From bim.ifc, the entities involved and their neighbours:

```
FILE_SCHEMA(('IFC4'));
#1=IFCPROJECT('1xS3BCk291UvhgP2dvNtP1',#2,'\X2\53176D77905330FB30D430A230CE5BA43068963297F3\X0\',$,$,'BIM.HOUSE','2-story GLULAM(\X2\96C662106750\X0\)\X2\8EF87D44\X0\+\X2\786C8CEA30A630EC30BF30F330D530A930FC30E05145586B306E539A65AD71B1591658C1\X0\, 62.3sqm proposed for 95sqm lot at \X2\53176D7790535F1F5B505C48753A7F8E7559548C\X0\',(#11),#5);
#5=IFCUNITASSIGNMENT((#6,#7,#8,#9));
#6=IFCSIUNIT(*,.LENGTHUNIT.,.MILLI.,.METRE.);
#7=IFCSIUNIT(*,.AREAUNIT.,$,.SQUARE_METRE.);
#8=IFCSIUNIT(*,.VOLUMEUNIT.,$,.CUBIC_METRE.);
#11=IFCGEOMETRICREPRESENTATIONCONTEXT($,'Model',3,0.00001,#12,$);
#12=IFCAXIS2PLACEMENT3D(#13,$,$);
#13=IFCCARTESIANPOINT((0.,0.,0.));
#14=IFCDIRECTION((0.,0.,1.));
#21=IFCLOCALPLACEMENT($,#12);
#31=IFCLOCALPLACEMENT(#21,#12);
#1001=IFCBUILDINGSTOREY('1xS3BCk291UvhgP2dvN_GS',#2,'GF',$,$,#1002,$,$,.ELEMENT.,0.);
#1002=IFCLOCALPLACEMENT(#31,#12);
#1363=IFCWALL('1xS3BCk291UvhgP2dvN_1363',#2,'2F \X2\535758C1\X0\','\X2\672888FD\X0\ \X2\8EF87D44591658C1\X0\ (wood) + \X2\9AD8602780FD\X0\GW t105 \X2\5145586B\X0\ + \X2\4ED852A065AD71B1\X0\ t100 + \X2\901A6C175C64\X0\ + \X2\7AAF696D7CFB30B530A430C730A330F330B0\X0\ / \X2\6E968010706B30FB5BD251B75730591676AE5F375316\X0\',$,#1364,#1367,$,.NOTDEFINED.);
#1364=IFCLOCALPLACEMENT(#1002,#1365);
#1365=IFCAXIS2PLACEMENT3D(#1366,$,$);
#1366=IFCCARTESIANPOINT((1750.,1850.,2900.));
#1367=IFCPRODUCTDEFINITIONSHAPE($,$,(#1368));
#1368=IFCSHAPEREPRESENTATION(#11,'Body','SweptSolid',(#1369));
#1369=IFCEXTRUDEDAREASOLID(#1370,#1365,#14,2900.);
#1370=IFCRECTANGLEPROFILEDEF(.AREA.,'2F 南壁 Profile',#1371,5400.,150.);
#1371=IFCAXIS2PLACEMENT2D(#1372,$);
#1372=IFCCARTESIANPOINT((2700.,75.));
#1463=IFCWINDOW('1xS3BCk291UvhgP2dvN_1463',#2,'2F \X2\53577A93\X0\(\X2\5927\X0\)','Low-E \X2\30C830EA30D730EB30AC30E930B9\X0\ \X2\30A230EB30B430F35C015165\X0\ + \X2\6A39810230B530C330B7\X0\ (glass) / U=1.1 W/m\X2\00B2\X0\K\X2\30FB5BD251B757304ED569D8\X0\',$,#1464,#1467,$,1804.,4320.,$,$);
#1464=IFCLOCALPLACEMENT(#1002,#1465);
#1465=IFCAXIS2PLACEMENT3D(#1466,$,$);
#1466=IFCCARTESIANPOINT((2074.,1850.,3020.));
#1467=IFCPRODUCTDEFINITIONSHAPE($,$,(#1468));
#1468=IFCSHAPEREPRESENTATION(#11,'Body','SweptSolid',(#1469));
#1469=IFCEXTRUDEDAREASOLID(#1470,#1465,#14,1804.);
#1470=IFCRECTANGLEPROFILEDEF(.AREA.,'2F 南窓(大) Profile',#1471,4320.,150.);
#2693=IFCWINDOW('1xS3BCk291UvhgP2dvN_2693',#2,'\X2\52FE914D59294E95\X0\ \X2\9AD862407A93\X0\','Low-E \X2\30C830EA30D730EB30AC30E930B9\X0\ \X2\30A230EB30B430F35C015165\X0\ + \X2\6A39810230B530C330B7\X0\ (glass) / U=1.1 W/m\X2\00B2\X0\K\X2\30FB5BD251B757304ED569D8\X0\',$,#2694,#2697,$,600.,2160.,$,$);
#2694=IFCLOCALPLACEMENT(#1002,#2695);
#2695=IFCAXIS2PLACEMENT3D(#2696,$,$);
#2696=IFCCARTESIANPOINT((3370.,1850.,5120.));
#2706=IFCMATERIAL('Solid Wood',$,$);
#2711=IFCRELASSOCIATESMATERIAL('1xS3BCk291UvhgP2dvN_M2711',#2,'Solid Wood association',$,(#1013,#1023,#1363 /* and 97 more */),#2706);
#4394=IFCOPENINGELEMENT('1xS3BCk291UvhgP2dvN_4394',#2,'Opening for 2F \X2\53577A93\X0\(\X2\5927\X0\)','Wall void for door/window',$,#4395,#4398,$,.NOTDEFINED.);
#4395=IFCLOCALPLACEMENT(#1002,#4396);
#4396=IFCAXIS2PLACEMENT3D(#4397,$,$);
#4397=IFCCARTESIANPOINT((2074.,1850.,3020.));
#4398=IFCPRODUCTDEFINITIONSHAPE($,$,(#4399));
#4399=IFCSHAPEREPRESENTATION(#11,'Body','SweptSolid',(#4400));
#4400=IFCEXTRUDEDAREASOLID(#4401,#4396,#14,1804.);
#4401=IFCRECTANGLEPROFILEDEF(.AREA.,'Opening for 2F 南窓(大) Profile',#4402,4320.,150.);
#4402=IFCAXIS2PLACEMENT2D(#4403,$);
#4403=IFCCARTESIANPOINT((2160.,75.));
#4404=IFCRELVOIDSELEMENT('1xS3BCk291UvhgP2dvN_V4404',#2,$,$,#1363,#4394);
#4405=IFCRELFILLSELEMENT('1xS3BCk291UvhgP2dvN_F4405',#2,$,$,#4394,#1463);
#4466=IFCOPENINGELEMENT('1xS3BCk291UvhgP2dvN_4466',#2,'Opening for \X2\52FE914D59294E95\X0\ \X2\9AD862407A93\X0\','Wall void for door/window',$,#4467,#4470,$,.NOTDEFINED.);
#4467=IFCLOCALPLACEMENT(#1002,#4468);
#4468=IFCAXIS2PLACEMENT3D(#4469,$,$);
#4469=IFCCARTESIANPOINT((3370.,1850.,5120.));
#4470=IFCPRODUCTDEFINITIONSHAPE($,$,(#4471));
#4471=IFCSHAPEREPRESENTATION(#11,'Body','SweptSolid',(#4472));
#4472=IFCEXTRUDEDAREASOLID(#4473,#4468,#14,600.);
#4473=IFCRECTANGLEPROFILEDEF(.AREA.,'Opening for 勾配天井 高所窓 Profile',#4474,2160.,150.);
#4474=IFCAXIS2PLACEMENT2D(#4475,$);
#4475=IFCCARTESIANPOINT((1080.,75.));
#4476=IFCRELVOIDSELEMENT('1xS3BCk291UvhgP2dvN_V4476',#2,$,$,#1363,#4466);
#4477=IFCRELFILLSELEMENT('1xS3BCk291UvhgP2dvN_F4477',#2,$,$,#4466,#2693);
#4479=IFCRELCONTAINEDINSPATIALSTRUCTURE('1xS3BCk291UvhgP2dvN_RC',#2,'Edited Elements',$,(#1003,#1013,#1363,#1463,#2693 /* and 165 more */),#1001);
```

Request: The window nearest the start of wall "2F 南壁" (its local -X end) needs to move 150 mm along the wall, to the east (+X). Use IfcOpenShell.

```python
import ifcopenshell
import ifcopenshell.api.geometry
import ifcopenshell.util.placement
import ifcopenshell.util.unit

model = ifcopenshell.open("bim.ifc")
unit_scale = ifcopenshell.util.unit.calculate_unit_scale(model)

window = model.by_guid("1xS3BCk291UvhgP2dvN_1463")
opening = window.FillsVoids[0].RelatingOpeningElement
wall = opening.VoidsElements[0].RelatingBuildingElement

wall_matrix = ifcopenshell.util.placement.get_local_placement(wall.ObjectPlacement)
shift = wall_matrix[:3, 0] * 0.15 / unit_scale
before = ifcopenshell.util.placement.get_local_placement(window.ObjectPlacement)[:3, 3].copy()

# The window is not placed relative to its opening, so move both.
for product in (opening, window):
    matrix = ifcopenshell.util.placement.get_local_placement(product.ObjectPlacement)
    matrix[:3, 3] += shift
    ifcopenshell.api.geometry.edit_object_placement(model, product=product, matrix=matrix, is_si=False)

after = ifcopenshell.util.placement.get_local_placement(window.ObjectPlacement)[:3, 3]
print("window moved by", (after - before).round(3) + 0.0)

model.write("bim_updated.ifc")
```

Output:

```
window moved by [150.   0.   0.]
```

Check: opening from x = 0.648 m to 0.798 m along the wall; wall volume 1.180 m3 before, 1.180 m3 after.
